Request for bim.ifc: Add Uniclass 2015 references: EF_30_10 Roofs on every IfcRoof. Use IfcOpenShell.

First a look at what the model holds.

```python
import ifcopenshell

model = ifcopenshell.open("bim.ifc")
print(model.schema)
print("classifications:", [c.Name for c in model.by_type("IfcClassification")])
for ifc_class in ("IfcDoor", "IfcRoof", "IfcStair", "IfcWall", "IfcWindow"):
    print(ifc_class, len(model.by_type(ifc_class)))
```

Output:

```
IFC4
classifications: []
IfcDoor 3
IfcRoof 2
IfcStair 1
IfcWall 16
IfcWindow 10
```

```python
import ifcopenshell
import ifcopenshell.api.classification

model = ifcopenshell.open("bim.ifc")

system = ifcopenshell.api.classification.add_classification(model, classification="Uniclass 2015")

codes = {
    "IfcRoof": ("EF_30_10", "Roofs"),
}
for ifc_class, (code, name) in codes.items():
    products = model.by_type(ifc_class)
    ifcopenshell.api.classification.add_reference(
        model, products=products, classification=system, identification=code, name=name
    )
    print(code, len(products))

model.write("bim_updated.ifc")
```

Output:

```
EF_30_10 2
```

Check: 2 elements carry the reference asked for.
